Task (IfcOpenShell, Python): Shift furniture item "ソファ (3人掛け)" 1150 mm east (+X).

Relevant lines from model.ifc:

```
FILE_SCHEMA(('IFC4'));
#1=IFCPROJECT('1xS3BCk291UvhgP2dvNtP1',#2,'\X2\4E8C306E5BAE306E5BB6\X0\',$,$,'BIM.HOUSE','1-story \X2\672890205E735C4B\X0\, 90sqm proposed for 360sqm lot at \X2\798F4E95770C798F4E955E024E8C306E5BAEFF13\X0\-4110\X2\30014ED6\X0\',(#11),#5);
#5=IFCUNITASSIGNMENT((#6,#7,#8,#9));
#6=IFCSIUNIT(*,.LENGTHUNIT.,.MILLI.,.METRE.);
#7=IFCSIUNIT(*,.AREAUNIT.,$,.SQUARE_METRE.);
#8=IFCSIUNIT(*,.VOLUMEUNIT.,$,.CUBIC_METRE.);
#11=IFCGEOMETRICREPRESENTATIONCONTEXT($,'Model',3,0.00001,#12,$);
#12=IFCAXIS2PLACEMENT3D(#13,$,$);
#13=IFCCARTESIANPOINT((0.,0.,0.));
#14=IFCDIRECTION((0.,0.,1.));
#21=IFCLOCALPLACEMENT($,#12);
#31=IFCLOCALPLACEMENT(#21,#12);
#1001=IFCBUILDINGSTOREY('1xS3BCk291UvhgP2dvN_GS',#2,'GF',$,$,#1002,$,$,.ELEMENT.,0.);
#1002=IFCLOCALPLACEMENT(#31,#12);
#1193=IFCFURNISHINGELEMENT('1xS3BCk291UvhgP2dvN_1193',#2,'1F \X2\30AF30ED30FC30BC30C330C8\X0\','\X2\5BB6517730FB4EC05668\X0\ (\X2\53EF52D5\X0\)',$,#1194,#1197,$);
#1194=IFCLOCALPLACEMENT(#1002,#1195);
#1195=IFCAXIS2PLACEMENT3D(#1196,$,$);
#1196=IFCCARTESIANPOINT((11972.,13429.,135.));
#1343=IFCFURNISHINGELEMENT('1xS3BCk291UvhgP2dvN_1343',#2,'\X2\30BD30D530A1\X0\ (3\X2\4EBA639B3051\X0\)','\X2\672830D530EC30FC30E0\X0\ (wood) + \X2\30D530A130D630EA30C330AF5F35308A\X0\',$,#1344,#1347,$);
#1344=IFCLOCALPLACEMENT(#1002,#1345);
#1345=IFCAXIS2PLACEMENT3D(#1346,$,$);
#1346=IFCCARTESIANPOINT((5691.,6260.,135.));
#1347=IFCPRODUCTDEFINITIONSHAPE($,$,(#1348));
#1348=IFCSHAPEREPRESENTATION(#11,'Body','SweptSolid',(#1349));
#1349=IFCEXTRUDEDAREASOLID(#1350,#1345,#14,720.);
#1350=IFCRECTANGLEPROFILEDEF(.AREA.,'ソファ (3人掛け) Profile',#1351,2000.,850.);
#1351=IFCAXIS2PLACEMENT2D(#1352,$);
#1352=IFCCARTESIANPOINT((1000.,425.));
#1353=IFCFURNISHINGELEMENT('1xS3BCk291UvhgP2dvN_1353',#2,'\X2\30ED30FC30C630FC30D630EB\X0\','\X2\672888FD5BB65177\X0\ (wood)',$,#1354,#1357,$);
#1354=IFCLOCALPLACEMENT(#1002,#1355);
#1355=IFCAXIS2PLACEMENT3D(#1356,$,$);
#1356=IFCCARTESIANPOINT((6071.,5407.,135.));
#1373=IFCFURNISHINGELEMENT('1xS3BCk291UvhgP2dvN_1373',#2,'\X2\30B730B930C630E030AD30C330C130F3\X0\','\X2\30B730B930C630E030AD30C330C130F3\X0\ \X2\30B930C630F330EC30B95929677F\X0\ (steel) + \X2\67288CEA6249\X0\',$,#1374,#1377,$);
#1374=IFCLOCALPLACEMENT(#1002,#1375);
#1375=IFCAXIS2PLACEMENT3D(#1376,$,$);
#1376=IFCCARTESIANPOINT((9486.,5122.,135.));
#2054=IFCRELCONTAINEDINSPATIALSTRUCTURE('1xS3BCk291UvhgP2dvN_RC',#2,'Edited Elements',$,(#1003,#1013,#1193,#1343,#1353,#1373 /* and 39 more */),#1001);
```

```python
import ifcopenshell
import ifcopenshell.api.geometry
import ifcopenshell.util.placement
import ifcopenshell.util.unit

model = ifcopenshell.open("model.ifc")
unit_scale = ifcopenshell.util.unit.calculate_unit_scale(model)

item = model.by_guid("1xS3BCk291UvhgP2dvN_1343")
matrix = ifcopenshell.util.placement.get_local_placement(item.ObjectPlacement)
matrix[0, 3] += 1.15 / unit_scale
ifcopenshell.api.geometry.edit_object_placement(model, product=item, matrix=matrix, is_si=False)

print(ifcopenshell.util.placement.get_local_placement(item.ObjectPlacement).round(3) + 0.0)

model.write("model-out.ifc")
```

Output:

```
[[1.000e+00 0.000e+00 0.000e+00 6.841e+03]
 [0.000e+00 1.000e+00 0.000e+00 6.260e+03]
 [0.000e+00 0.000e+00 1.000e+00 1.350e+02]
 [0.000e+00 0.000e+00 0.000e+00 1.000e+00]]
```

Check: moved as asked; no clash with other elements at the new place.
